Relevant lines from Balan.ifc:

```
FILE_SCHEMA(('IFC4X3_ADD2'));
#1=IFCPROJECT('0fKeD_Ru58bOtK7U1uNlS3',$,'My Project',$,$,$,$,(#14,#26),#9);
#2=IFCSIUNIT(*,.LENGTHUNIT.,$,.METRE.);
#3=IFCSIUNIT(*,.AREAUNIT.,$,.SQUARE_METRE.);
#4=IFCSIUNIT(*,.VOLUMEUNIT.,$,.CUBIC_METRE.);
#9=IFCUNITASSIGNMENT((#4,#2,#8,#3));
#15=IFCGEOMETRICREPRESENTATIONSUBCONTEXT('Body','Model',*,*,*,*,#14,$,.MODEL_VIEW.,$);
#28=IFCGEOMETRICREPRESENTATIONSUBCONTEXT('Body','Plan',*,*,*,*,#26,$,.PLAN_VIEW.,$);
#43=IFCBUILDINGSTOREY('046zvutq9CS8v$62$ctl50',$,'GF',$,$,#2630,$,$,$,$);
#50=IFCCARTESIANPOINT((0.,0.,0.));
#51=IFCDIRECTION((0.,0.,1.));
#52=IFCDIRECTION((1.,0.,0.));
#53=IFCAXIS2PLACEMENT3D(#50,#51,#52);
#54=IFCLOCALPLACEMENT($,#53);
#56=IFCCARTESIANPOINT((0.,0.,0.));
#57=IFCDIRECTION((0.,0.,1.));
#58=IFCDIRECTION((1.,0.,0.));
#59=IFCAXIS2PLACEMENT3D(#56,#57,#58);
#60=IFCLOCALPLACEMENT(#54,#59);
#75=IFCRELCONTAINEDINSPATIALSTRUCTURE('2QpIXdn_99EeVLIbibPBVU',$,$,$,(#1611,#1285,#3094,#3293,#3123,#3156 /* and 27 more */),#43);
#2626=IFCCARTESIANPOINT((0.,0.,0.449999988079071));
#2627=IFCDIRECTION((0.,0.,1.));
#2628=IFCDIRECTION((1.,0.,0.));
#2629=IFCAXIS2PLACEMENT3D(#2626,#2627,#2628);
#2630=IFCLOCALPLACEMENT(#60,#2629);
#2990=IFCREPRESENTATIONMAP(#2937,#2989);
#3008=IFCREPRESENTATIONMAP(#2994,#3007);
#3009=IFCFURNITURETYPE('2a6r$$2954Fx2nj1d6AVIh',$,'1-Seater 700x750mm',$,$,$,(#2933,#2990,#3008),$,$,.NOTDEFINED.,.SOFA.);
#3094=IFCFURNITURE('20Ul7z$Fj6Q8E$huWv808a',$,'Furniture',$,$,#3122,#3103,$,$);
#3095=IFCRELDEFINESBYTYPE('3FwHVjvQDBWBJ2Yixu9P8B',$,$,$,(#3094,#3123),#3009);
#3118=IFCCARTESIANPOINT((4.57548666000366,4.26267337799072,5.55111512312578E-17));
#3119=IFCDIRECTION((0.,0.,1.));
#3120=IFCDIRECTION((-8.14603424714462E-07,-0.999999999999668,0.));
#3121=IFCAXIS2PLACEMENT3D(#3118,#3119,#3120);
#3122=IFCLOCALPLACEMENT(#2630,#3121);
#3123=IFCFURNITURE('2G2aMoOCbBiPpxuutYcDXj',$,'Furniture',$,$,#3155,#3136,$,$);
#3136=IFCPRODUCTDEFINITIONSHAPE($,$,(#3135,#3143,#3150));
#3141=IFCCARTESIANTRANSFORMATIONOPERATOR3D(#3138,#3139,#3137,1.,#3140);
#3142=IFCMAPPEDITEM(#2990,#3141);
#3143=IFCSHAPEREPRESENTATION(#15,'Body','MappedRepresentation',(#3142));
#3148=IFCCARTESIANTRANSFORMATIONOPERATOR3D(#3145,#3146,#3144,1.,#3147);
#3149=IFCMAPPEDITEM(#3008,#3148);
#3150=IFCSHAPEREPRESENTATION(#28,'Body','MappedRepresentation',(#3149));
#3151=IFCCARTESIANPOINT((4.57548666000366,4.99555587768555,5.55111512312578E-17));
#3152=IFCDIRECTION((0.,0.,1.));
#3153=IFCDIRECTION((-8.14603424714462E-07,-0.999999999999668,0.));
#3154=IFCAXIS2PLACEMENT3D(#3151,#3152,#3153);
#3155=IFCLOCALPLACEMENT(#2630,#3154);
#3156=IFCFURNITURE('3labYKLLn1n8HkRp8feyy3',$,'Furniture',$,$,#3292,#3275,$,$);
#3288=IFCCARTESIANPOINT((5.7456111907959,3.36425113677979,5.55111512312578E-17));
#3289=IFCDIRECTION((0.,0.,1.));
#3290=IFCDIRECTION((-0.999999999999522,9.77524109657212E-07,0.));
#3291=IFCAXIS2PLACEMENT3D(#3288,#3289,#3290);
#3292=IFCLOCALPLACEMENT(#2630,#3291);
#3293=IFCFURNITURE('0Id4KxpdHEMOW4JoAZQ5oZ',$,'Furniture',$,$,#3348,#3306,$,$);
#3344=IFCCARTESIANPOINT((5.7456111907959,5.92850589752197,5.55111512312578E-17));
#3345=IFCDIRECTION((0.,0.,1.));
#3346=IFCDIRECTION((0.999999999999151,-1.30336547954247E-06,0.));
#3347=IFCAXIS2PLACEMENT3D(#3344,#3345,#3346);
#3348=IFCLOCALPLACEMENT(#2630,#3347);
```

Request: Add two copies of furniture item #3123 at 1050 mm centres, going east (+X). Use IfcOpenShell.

```python
import numpy as np
import ifcopenshell
import ifcopenshell.api.geometry
import ifcopenshell.api.root
import ifcopenshell.util.element
import ifcopenshell.util.placement
import ifcopenshell.util.unit

model = ifcopenshell.open("Balan.ifc")
unit_scale = ifcopenshell.util.unit.calculate_unit_scale(model)

source = model.by_id(3123)
base = ifcopenshell.util.placement.get_local_placement(source.ObjectPlacement)
step = np.array([1.0, 0.0, 0.0]) * 1.05 / unit_scale

for i in range(1, 3):
    copy = ifcopenshell.api.root.copy_class(model, product=source)
    copy.Representation = ifcopenshell.util.element.copy_deep(
        model, source.Representation, exclude=["IfcGeometricRepresentationContext", "IfcRepresentationMap"]
    )
    matrix = base.copy()
    matrix[:3, 3] += i * step
    print("added at", matrix[:3, 3].round(3) + 0.0)
    ifcopenshell.api.geometry.edit_object_placement(model, product=copy, matrix=matrix, is_si=False)

model.write("Balan-out.ifc")
```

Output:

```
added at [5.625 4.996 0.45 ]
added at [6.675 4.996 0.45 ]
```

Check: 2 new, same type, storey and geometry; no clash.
